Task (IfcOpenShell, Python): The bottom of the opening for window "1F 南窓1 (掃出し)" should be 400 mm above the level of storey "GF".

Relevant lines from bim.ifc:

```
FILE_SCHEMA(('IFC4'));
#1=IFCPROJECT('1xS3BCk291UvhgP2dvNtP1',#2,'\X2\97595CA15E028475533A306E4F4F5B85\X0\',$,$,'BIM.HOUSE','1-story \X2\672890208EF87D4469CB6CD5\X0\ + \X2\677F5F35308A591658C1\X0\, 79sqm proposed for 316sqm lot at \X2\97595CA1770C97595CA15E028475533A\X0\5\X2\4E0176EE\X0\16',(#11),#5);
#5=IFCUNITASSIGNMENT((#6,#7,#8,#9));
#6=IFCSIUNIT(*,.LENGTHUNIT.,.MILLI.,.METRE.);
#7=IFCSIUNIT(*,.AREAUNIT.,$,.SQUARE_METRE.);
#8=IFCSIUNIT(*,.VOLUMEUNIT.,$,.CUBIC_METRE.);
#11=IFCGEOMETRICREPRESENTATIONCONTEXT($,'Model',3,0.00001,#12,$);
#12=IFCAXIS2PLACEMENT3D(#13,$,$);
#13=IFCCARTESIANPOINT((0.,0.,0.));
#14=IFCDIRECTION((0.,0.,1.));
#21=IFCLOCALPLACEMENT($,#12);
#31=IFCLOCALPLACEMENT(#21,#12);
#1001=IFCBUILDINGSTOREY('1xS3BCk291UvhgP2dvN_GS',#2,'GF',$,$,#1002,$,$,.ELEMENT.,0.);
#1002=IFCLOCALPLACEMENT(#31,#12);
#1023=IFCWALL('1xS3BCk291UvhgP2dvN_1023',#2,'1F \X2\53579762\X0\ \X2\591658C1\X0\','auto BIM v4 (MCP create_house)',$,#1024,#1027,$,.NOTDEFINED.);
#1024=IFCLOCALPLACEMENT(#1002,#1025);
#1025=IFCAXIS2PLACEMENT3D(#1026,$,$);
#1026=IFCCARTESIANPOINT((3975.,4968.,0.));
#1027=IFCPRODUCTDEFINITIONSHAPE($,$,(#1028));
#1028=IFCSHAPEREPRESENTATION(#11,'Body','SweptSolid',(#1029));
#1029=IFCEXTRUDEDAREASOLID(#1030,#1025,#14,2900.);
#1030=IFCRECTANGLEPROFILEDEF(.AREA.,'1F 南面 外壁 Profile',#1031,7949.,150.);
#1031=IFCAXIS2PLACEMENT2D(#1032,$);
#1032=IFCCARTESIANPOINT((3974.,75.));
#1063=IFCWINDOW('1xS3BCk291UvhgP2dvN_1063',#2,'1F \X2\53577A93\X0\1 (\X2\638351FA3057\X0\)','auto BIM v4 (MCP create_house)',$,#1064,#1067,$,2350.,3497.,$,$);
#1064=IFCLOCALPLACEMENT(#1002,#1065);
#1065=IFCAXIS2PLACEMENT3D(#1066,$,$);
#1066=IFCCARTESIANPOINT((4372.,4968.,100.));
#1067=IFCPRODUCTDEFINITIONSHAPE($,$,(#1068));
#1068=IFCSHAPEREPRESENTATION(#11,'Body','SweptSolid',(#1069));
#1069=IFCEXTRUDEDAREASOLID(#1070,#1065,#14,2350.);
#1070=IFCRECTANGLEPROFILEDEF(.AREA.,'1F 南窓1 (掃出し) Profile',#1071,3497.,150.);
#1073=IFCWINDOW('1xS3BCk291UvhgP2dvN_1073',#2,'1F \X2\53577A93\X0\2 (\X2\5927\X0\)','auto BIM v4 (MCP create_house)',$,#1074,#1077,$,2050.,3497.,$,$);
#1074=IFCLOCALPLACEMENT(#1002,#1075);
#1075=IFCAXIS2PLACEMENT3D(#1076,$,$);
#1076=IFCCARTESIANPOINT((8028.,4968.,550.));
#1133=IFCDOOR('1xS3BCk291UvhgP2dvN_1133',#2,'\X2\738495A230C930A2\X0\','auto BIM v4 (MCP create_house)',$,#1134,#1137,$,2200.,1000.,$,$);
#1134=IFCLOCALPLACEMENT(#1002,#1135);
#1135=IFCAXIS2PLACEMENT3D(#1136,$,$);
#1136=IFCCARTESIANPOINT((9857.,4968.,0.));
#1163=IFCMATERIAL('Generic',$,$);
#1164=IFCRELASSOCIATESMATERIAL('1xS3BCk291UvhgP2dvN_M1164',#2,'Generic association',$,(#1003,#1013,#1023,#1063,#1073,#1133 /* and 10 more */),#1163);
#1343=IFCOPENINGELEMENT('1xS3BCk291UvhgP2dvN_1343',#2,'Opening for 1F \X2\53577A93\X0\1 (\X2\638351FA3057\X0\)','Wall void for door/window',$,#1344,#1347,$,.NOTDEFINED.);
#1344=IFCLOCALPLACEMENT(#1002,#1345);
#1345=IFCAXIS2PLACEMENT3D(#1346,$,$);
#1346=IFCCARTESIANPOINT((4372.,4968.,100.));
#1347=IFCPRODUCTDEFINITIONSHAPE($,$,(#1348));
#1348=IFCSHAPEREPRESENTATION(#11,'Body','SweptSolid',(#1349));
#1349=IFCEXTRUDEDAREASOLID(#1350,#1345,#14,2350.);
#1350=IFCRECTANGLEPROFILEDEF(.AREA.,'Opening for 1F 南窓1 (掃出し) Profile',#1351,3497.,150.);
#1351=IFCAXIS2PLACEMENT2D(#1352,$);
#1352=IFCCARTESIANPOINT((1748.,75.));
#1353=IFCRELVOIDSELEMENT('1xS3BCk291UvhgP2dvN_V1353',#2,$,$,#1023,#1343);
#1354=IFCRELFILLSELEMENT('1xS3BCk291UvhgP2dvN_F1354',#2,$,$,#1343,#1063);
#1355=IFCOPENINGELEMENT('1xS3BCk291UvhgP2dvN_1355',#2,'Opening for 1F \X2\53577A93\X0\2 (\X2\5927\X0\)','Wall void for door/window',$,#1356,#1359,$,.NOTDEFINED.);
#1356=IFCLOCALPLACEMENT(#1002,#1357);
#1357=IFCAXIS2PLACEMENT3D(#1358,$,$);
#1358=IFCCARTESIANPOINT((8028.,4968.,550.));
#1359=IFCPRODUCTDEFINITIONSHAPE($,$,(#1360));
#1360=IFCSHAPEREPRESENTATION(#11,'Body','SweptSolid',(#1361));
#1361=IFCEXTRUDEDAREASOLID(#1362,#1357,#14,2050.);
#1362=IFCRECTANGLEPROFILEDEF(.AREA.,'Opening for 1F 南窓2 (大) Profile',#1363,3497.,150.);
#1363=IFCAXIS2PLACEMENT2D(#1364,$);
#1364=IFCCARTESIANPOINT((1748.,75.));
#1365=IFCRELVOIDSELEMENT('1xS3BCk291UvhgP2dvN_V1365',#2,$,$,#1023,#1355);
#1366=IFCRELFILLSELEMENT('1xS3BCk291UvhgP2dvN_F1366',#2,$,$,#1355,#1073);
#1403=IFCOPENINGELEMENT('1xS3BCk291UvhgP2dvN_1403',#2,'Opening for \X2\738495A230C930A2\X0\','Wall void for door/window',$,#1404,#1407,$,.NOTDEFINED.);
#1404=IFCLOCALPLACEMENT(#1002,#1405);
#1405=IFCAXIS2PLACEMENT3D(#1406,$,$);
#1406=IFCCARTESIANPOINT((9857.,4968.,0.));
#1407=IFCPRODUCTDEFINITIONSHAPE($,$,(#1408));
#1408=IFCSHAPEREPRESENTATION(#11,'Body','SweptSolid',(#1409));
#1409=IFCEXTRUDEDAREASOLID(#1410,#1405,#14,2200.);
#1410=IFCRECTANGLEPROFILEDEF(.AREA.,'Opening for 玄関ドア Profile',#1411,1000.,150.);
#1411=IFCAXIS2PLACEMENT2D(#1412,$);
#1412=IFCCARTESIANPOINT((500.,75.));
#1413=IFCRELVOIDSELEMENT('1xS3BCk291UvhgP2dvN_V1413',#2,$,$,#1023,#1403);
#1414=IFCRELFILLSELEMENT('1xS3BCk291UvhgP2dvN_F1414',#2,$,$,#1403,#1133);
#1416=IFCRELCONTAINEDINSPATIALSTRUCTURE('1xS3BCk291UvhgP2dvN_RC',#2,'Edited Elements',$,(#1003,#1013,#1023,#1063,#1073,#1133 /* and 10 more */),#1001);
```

```python
import numpy as np
import ifcopenshell
import ifcopenshell.api.geometry
import ifcopenshell.geom
import ifcopenshell.util.element
import ifcopenshell.util.placement
import ifcopenshell.util.shape
import ifcopenshell.util.unit

model = ifcopenshell.open("bim.ifc")
unit_scale = ifcopenshell.util.unit.calculate_unit_scale(model)

window = model.by_guid("1xS3BCk291UvhgP2dvN_1063")
opening = window.FillsVoids[0].RelatingOpeningElement
storey = ifcopenshell.util.element.get_container(window, ifc_class="IfcBuildingStorey")
level = ifcopenshell.util.placement.get_local_placement(storey.ObjectPlacement)[2, 3]

# The opening's origin need not be at the sill, so measure its lowest point.
shape = ifcopenshell.geom.create_shape(ifcopenshell.geom.settings(), opening)
bottom = ifcopenshell.util.shape.get_shape_bottom_elevation(shape, shape.geometry) / unit_scale
dz = level + 400.0 - bottom

shift = np.array([0.0, 0.0, dz])
# The window is not placed relative to its opening, so move both.
for product in (opening, window):
    matrix = ifcopenshell.util.placement.get_local_placement(product.ObjectPlacement)
    matrix[:3, 3] += shift
    ifcopenshell.api.geometry.edit_object_placement(model, product=product, matrix=matrix, is_si=False)

print(f"moved by {dz * unit_scale:+.3f} m")

model.write("bim-out.ifc")
```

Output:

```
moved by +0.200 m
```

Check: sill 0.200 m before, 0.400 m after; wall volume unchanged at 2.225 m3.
